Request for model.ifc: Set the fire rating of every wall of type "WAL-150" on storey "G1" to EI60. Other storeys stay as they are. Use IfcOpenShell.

First a look at what the model holds.

```python
import ifcopenshell
import ifcopenshell.util.element

model = ifcopenshell.open("model.ifc")
print(model.schema)
storey = next(s for s in model.by_type("IfcBuildingStorey") if s.Name == "G1")
walls = [e for e in ifcopenshell.util.element.get_decomposition(storey) if e.is_a("IfcWall")]
seen = {}
for e in walls:
    element_type = ifcopenshell.util.element.get_type(e)
    key = (element_type.Name if element_type != e and element_type else None, ifcopenshell.util.element.get_pset(e, "Pset_WallCommon", "FireRating"))
    seen[key] = seen.get(key, 0) + 1
for (name, value), count in sorted(seen.items(), key=str):
    print(count, "x", name, "|", value)
```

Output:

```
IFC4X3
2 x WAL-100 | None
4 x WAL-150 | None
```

```python
import ifcopenshell
import ifcopenshell.api.pset
import ifcopenshell.util.element

model = ifcopenshell.open("model.ifc")

storey = next(s for s in model.by_type("IfcBuildingStorey") if s.Name == "G1")
walls = [e for e in ifcopenshell.util.element.get_decomposition(storey) if e.is_a("IfcWall")]

count = 0
for e in walls:
    element_type = ifcopenshell.util.element.get_type(e)
    if element_type in (None, e) or element_type.Name != "WAL-150":
        continue
    # add_pset returns the element's existing set when there is one.
    pset = ifcopenshell.api.pset.add_pset(model, product=e, name="Pset_WallCommon")
    ifcopenshell.api.pset.edit_pset(model, pset=pset, properties={"FireRating": "EI60"})
    count += 1

print(count, "walls updated")

model.write("model_edited.ifc")
```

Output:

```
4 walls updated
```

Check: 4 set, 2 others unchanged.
